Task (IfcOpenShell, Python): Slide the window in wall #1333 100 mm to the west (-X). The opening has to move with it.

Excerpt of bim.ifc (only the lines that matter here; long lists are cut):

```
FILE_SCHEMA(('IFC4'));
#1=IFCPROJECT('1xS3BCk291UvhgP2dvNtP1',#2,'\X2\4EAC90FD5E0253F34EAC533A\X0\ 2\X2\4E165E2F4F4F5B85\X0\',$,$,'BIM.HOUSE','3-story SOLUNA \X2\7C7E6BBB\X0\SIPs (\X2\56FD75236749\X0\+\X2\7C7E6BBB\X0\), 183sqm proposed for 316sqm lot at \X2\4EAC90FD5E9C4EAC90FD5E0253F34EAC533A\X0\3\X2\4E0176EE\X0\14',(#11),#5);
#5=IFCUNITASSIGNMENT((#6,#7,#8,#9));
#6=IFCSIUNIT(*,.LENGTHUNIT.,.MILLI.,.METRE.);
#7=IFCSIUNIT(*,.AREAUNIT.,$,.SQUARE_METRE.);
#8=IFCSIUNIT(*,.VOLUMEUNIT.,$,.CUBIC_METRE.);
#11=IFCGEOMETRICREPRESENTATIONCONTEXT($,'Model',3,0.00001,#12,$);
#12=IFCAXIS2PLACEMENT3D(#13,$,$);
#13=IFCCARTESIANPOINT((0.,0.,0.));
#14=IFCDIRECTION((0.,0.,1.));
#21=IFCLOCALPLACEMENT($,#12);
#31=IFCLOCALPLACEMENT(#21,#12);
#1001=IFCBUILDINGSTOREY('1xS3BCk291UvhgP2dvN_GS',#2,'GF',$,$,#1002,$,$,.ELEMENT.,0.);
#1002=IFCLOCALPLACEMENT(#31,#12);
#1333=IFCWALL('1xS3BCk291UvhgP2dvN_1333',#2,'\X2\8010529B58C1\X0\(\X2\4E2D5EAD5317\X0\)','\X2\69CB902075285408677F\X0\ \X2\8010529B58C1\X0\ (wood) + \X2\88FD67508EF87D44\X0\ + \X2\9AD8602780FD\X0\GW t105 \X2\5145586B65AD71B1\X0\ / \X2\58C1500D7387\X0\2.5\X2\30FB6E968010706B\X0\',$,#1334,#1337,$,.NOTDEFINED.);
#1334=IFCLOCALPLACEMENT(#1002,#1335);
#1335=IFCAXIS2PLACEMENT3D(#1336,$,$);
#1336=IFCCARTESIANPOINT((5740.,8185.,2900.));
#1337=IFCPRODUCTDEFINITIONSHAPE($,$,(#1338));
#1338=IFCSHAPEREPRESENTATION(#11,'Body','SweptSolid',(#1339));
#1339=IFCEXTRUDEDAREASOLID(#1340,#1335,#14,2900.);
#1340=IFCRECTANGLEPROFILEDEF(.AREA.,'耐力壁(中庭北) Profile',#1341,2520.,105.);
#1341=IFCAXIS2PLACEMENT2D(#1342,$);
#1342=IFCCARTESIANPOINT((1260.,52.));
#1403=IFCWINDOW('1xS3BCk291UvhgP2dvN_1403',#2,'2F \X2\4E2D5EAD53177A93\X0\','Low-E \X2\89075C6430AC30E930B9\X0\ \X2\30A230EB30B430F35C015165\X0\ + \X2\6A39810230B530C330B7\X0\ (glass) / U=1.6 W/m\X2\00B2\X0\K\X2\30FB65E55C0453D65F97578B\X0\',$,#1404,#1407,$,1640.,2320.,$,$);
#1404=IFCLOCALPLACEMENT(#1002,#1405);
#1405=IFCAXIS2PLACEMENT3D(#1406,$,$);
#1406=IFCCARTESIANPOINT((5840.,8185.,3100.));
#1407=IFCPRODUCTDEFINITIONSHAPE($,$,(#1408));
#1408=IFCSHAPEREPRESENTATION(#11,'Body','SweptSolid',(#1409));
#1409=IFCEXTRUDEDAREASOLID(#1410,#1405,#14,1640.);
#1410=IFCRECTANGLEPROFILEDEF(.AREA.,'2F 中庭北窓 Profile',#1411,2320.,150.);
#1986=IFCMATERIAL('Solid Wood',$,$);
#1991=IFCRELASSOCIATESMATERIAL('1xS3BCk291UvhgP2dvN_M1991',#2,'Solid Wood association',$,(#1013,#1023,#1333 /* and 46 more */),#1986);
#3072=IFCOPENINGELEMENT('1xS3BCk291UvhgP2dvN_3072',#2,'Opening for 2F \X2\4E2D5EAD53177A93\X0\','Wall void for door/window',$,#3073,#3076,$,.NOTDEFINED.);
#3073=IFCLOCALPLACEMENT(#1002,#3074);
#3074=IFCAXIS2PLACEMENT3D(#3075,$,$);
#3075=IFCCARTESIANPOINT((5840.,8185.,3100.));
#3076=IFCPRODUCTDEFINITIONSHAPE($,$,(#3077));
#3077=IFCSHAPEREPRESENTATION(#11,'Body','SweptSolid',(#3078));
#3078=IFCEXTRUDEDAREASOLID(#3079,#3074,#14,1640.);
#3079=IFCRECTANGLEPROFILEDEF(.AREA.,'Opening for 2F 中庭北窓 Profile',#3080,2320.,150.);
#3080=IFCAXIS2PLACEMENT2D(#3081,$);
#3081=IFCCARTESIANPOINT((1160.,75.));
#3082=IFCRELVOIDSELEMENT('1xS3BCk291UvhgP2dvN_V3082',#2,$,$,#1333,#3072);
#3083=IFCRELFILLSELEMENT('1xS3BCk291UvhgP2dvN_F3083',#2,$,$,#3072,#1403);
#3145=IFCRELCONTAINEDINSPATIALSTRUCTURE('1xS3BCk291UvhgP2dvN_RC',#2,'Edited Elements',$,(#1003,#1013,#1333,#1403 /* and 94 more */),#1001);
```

```python
import ifcopenshell
import ifcopenshell.api.geometry
import ifcopenshell.util.placement
import ifcopenshell.util.unit

model = ifcopenshell.open("bim.ifc")
unit_scale = ifcopenshell.util.unit.calculate_unit_scale(model)

window = model.by_guid("1xS3BCk291UvhgP2dvN_1403")
opening = window.FillsVoids[0].RelatingOpeningElement
wall = opening.VoidsElements[0].RelatingBuildingElement

wall_matrix = ifcopenshell.util.placement.get_local_placement(wall.ObjectPlacement)
shift = wall_matrix[:3, 0] * -0.1 / unit_scale
before = ifcopenshell.util.placement.get_local_placement(window.ObjectPlacement)[:3, 3].copy()

# The window is not placed relative to its opening, so move both.
for product in (opening, window):
    matrix = ifcopenshell.util.placement.get_local_placement(product.ObjectPlacement)
    matrix[:3, 3] += shift
    ifcopenshell.api.geometry.edit_object_placement(model, product=product, matrix=matrix, is_si=False)

after = ifcopenshell.util.placement.get_local_placement(window.ObjectPlacement)[:3, 3]
print("window moved by", (after - before).round(3) + 0.0)

model.write("bim_v2.ifc")
```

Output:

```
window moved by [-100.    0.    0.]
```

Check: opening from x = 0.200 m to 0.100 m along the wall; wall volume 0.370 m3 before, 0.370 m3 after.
